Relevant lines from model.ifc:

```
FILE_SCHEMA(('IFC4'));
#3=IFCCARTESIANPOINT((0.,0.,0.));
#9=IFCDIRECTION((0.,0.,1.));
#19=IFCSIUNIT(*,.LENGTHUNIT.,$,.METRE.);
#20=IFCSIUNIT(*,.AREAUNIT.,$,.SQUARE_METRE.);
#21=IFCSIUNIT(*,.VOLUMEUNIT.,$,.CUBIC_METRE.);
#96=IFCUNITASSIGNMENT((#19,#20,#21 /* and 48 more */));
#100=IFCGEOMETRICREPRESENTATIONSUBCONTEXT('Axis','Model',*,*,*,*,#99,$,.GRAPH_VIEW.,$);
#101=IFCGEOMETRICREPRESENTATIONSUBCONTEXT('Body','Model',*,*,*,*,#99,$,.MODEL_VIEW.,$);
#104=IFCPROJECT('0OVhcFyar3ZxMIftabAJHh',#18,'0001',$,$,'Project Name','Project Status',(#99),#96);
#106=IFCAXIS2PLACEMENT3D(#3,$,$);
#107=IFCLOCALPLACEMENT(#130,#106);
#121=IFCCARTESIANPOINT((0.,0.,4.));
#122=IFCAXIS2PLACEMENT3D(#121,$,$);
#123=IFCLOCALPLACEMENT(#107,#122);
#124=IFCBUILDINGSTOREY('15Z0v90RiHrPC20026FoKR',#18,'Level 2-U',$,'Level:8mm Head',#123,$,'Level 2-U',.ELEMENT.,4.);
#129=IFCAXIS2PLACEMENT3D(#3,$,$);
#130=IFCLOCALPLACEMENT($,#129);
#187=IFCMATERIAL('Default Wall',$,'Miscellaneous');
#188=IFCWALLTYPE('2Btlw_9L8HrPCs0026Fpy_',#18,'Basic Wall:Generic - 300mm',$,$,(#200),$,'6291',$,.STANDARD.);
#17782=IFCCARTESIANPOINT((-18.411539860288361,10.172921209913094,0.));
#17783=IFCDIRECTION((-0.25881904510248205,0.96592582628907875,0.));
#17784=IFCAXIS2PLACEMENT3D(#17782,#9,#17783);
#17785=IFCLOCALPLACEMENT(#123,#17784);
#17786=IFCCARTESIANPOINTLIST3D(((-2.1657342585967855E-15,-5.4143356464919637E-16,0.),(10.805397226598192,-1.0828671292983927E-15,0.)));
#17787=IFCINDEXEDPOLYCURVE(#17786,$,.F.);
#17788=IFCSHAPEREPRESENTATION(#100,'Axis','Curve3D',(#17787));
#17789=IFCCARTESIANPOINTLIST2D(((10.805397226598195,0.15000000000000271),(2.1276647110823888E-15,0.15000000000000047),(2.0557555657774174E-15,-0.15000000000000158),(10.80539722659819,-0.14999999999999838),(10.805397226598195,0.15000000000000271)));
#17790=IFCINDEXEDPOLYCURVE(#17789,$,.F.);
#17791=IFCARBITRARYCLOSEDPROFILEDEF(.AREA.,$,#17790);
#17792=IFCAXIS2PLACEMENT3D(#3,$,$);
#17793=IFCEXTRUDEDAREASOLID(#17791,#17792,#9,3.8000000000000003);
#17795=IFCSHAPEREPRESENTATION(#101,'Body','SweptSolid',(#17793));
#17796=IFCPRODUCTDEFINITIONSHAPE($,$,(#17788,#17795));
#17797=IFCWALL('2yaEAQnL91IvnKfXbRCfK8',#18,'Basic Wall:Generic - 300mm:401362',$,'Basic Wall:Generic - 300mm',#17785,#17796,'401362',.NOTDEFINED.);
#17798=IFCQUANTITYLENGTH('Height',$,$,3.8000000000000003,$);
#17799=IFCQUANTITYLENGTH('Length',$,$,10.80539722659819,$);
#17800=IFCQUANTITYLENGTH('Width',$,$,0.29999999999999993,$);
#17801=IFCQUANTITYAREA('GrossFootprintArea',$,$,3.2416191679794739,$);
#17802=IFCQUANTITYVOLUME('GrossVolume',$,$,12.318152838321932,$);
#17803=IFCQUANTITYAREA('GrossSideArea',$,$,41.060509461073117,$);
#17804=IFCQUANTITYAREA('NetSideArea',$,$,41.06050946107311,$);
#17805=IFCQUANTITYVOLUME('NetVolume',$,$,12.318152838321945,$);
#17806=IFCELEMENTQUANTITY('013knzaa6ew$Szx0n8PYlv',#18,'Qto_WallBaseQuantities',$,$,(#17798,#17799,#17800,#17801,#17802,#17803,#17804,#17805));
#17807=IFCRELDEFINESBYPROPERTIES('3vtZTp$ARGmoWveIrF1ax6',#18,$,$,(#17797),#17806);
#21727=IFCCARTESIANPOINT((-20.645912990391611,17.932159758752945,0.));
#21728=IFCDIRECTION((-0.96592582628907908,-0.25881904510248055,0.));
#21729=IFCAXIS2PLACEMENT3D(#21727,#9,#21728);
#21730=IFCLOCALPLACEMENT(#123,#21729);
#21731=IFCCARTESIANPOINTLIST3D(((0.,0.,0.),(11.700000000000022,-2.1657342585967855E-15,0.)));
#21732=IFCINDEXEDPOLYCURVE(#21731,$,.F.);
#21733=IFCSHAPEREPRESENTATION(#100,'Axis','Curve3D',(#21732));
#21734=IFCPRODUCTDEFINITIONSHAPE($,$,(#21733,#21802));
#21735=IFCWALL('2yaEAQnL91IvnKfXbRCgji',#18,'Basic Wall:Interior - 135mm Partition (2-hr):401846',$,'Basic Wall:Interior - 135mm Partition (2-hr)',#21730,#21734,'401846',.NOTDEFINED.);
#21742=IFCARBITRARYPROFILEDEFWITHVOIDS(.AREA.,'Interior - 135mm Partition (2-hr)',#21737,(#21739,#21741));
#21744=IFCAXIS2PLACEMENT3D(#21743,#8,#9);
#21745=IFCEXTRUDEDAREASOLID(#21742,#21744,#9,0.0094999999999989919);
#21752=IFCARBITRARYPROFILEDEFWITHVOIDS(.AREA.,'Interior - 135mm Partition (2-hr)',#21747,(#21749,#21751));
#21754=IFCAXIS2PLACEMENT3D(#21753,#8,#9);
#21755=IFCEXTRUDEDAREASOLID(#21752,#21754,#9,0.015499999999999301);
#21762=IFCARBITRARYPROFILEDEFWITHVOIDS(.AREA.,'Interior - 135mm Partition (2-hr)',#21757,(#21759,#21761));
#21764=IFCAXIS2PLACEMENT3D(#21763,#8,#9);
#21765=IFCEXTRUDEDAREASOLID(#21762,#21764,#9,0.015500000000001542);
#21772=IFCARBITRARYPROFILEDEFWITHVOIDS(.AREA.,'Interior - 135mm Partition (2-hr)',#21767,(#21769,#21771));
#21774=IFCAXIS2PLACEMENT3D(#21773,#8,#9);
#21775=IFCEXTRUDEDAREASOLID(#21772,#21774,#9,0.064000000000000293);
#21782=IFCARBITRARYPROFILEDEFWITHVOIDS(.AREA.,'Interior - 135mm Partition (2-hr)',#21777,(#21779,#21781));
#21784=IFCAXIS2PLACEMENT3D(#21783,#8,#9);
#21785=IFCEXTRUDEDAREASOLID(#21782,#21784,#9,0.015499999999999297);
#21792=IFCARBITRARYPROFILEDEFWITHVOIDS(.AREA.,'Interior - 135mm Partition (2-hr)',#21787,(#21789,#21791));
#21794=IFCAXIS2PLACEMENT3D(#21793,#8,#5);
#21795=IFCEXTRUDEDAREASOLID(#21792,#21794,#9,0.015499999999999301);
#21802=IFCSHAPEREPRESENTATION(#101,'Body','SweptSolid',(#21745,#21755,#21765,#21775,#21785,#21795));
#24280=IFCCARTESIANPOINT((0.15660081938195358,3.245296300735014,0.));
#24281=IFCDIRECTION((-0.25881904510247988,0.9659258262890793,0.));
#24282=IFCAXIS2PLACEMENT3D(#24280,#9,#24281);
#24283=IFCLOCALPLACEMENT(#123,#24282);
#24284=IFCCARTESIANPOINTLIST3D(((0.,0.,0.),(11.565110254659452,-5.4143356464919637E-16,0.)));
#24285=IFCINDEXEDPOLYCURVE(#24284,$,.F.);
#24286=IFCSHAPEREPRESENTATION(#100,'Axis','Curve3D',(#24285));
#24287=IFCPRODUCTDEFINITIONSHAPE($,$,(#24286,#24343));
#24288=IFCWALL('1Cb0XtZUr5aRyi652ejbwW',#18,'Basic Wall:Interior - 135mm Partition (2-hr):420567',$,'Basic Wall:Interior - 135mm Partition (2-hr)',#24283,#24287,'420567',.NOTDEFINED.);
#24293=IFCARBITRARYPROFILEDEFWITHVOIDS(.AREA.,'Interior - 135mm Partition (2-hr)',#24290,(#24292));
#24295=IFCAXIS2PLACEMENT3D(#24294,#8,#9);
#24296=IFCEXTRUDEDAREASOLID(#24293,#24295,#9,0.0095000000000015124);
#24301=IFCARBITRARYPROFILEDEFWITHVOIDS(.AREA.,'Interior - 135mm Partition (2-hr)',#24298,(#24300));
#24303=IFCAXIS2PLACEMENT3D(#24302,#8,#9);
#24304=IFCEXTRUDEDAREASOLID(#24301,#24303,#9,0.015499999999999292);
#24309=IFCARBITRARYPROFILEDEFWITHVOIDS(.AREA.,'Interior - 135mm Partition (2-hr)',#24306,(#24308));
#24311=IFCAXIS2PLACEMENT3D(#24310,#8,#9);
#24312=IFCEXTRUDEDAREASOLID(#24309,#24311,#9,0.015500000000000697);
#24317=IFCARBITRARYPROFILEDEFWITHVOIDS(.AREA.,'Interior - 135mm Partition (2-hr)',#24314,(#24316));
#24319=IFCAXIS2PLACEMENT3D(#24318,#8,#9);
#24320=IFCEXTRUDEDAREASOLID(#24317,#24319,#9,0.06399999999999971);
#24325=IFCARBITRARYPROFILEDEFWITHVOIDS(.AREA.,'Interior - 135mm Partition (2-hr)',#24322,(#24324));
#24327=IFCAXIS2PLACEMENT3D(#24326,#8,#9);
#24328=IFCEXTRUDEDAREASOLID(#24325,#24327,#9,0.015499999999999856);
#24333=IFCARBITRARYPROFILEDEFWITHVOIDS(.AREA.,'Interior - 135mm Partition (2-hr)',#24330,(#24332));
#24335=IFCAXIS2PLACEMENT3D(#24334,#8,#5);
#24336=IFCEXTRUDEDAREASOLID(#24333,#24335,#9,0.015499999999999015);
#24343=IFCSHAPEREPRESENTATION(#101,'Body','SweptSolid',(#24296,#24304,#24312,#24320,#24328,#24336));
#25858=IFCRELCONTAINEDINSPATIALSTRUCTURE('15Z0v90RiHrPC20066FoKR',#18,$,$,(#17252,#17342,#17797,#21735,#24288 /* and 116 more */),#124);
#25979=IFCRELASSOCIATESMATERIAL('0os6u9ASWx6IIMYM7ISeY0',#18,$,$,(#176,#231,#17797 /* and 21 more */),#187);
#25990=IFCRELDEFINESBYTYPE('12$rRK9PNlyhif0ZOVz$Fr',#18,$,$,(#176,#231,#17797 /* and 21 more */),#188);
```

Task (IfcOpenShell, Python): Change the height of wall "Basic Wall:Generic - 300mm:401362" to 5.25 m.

```python
import ifcopenshell
import ifcopenshell.api.pset
import ifcopenshell.geom
import ifcopenshell.util.element
import ifcopenshell.util.representation
import ifcopenshell.util.shape
import ifcopenshell.util.unit

model = ifcopenshell.open("model.ifc")
unit_scale = ifcopenshell.util.unit.calculate_unit_scale(model)
area_scale = ifcopenshell.util.unit.calculate_unit_scale(model, "AREAUNIT")
volume_scale = ifcopenshell.util.unit.calculate_unit_scale(model, "VOLUMEUNIT")
settings = ifcopenshell.geom.settings()


def volume(element):
    """Net volume in cubic metres, openings subtracted."""
    shape = ifcopenshell.geom.create_shape(settings, element)
    return ifcopenshell.util.shape.get_volume(shape.geometry)


wall = model.by_guid("2yaEAQnL91IvnKfXbRCfK8")
before = volume(wall)

body = ifcopenshell.util.representation.get_representation(wall, "Model", "Body")
solid = body.Items[0]
old_height = solid.Depth
solid.Depth = 5.25 / unit_scale
after = volume(wall)
thickness = 0.3  # wall thickness in metres

# Update the stored height, areas and volumes.
qto = model.by_id(ifcopenshell.util.element.get_pset(wall, "Qto_WallBaseQuantities", should_inherit=False)["id"])
ifcopenshell.api.pset.edit_qto(model, qto=qto, properties={
    "Height": solid.Depth,
    "GrossVolume": ifcopenshell.util.element.get_pset(wall, "Qto_WallBaseQuantities", "GrossVolume") * solid.Depth / old_height,
    "GrossSideArea": ifcopenshell.util.element.get_pset(wall, "Qto_WallBaseQuantities", "GrossSideArea") * solid.Depth / old_height,
    "NetSideArea": after / thickness / area_scale,
    "NetVolume": after / volume_scale,
})

print(f"height {old_height:g} -> {solid.Depth:g}, volume {before:.3f} -> {after:.3f} m3")

model.write("model_v2.ifc")
```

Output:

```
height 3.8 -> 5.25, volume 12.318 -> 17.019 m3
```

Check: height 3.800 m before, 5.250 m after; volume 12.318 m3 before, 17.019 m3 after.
